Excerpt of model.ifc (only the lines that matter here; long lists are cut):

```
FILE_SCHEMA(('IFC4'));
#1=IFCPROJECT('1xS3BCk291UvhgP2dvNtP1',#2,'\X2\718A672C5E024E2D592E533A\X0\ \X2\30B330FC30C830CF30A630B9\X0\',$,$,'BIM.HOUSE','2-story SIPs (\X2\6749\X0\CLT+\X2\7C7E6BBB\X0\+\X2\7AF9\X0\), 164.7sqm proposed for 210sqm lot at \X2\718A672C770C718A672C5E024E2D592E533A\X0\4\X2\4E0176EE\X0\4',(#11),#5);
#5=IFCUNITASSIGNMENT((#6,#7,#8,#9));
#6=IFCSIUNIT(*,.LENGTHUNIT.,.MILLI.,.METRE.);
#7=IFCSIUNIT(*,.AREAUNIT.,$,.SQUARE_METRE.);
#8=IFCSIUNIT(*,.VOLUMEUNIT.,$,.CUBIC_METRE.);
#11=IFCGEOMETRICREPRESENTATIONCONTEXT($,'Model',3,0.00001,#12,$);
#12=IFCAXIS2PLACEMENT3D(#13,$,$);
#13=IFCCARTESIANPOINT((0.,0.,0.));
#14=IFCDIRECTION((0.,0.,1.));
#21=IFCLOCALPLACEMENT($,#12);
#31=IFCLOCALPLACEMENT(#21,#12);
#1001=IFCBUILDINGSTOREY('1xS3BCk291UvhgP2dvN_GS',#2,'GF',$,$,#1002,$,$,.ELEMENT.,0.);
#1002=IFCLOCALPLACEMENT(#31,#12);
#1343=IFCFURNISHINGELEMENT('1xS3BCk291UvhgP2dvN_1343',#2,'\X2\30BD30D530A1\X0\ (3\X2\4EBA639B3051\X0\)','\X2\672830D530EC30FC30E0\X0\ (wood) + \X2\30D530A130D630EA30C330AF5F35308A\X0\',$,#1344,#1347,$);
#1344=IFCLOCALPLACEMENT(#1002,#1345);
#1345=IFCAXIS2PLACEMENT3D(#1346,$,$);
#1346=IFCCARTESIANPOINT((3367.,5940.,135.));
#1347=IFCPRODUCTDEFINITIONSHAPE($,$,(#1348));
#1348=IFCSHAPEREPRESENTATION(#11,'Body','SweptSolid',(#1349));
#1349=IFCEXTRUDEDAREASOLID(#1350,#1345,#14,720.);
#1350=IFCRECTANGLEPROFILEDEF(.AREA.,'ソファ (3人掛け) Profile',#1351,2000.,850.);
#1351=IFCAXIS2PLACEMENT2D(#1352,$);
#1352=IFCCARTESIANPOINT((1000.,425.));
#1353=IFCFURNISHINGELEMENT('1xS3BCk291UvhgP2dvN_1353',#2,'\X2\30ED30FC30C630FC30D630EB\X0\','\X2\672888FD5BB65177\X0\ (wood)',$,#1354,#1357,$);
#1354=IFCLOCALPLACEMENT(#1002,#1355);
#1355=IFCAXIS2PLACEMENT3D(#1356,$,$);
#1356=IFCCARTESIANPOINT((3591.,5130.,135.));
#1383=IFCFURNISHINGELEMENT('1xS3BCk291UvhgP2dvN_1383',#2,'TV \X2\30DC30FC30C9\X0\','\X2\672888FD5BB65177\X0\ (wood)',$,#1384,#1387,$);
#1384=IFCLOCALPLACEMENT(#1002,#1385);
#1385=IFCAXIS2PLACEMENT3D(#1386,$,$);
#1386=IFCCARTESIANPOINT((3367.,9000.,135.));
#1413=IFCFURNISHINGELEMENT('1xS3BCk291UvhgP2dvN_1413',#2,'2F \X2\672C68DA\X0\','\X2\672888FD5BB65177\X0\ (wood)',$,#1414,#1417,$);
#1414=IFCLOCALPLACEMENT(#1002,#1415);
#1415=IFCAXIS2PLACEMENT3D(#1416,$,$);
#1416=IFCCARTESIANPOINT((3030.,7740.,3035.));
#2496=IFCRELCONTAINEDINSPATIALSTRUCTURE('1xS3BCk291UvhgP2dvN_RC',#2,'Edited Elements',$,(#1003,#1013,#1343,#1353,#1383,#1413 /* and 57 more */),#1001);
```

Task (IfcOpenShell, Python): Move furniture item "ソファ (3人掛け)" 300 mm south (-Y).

```python
import ifcopenshell
import ifcopenshell.api.geometry
import ifcopenshell.util.placement
import ifcopenshell.util.unit

model = ifcopenshell.open("model.ifc")
unit_scale = ifcopenshell.util.unit.calculate_unit_scale(model)

item = model.by_guid("1xS3BCk291UvhgP2dvN_1343")
matrix = ifcopenshell.util.placement.get_local_placement(item.ObjectPlacement)
matrix[1, 3] -= 0.3 / unit_scale
ifcopenshell.api.geometry.edit_object_placement(model, product=item, matrix=matrix, is_si=False)

print(ifcopenshell.util.placement.get_local_placement(item.ObjectPlacement).round(3) + 0.0)

model.write("model-out.ifc")
```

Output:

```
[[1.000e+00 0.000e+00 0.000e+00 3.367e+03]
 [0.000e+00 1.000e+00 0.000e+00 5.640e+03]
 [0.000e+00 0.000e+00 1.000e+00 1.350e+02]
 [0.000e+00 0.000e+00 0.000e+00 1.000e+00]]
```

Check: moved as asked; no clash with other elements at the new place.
